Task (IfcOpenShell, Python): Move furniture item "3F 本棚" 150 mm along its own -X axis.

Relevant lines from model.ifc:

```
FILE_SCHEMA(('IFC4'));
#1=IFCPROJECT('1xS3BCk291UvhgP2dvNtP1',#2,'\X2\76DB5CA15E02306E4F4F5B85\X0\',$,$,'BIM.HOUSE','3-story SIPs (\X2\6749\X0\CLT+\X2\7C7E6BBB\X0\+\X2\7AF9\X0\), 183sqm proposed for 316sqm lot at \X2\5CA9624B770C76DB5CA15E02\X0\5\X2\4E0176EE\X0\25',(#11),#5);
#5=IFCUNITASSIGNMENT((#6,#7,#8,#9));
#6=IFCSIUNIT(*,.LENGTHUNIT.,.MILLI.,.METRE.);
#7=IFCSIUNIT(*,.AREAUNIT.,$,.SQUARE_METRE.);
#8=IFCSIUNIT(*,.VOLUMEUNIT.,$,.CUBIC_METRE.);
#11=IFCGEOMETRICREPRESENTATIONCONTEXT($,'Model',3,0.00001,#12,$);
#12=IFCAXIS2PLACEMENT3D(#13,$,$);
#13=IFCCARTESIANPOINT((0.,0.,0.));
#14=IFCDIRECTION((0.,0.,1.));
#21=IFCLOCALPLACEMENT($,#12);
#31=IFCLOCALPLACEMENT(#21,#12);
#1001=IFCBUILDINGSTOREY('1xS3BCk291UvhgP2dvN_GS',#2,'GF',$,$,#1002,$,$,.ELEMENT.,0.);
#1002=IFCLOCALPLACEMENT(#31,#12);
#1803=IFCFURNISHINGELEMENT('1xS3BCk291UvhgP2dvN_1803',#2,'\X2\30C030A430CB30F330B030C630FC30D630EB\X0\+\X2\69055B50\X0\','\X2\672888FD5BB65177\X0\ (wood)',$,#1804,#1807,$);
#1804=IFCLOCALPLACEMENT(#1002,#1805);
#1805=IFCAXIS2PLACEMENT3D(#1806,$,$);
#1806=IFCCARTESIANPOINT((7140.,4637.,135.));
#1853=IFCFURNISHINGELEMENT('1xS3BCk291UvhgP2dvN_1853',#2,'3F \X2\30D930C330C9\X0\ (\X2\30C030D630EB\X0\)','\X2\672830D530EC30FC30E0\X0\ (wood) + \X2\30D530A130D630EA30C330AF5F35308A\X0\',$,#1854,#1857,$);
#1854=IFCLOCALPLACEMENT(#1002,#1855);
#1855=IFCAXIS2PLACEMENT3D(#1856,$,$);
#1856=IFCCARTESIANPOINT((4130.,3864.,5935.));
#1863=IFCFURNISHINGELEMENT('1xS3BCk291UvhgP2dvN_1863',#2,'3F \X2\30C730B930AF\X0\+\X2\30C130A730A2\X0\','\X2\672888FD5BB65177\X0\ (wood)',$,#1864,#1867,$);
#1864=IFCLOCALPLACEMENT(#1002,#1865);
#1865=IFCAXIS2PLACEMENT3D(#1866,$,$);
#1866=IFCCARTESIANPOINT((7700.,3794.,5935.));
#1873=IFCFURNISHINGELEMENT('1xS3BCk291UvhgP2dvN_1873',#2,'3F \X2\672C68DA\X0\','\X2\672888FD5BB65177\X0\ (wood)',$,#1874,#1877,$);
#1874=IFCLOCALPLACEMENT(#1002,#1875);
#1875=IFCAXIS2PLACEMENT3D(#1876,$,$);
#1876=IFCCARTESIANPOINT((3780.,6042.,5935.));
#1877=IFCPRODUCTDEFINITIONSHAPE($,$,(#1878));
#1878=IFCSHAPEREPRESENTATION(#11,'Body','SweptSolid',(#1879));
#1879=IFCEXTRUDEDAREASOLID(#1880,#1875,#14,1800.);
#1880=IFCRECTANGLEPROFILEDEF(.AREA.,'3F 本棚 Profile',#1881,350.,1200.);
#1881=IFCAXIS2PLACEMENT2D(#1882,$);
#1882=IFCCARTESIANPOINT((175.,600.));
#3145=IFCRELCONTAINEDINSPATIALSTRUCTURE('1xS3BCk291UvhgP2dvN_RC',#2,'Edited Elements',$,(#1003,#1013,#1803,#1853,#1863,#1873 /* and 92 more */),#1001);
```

```python
import ifcopenshell
import ifcopenshell.api.geometry
import ifcopenshell.util.placement

model = ifcopenshell.open("model.ifc")

item = model.by_guid("1xS3BCk291UvhgP2dvN_1873")
matrix = ifcopenshell.util.placement.get_local_placement(item.ObjectPlacement)
matrix[:3, 3] -= matrix[:3, 0] * 150.0
ifcopenshell.api.geometry.edit_object_placement(model, product=item, matrix=matrix, is_si=False)

print(ifcopenshell.util.placement.get_local_placement(item.ObjectPlacement).round(3) + 0.0)

model.write("model_v2.ifc")
```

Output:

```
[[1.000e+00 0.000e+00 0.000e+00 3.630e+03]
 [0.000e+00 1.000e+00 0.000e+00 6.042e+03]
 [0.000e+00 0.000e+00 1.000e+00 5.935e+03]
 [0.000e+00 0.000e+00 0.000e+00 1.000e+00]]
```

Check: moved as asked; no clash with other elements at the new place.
